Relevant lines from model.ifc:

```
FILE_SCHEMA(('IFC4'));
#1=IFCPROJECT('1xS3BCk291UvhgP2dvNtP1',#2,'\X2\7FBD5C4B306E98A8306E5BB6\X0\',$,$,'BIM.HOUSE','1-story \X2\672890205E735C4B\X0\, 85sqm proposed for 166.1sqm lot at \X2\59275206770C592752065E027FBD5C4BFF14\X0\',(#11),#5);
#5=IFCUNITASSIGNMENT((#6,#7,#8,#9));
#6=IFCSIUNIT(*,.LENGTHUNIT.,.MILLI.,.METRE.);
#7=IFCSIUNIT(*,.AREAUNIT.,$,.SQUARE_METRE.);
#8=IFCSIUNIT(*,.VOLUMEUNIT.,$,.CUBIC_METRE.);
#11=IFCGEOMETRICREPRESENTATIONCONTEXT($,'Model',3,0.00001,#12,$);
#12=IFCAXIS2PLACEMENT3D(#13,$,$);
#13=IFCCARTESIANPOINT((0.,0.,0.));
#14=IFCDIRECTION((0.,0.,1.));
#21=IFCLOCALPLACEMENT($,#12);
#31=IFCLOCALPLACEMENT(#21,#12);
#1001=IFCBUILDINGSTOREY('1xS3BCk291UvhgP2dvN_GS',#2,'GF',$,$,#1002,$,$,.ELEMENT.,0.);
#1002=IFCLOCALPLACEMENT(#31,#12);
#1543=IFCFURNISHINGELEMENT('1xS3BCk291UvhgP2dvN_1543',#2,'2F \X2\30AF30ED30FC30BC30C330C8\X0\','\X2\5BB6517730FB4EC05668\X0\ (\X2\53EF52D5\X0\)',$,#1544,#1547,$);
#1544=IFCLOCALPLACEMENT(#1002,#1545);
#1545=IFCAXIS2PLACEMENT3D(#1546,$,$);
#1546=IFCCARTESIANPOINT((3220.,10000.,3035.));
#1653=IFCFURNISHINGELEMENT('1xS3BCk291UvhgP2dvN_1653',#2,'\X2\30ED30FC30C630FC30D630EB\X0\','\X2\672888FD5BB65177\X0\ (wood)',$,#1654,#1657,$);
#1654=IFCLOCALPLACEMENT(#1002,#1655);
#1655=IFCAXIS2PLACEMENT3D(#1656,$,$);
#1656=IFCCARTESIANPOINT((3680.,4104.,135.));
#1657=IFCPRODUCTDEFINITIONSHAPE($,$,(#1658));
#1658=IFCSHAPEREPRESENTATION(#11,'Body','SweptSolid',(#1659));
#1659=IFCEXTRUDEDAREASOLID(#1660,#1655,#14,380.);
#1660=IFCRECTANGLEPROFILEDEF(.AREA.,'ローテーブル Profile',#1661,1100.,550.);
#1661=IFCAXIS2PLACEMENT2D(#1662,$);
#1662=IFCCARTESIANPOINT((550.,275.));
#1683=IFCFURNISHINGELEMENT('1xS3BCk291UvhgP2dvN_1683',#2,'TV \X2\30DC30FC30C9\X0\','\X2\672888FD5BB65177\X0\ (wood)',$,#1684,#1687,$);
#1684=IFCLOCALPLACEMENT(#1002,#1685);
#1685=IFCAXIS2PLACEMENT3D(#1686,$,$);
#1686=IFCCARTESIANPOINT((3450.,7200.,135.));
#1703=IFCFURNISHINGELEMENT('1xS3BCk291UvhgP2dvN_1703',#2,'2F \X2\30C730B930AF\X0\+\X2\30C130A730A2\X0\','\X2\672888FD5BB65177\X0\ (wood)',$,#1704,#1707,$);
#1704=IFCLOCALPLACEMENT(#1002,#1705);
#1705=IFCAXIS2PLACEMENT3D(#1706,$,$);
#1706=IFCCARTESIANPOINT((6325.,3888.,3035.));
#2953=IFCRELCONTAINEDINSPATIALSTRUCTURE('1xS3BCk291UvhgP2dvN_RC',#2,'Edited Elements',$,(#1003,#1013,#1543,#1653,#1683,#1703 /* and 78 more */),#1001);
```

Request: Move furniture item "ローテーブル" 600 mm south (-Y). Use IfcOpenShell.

```python
import ifcopenshell
import ifcopenshell.api.geometry
import ifcopenshell.util.placement

model = ifcopenshell.open("model.ifc")

item = model.by_id(1653)
matrix = ifcopenshell.util.placement.get_local_placement(item.ObjectPlacement)
matrix[1, 3] -= 600.0
ifcopenshell.api.geometry.edit_object_placement(model, product=item, matrix=matrix, is_si=False)

print(ifcopenshell.util.placement.get_local_placement(item.ObjectPlacement).round(3) + 0.0)

model.write("model_rev.ifc")
```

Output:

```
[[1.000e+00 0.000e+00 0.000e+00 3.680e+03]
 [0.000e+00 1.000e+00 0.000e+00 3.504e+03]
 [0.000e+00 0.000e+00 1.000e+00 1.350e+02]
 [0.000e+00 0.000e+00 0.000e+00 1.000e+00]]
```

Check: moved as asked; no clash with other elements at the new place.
